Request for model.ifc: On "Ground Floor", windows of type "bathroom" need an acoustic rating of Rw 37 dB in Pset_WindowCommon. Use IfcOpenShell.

First a look at what the model holds.

```python
import ifcopenshell
import ifcopenshell.util.element

model = ifcopenshell.open("model.ifc")
print(model.schema)
storey = next(s for s in model.by_type("IfcBuildingStorey") if s.Name == "Ground Floor")
windows = [e for e in ifcopenshell.util.element.get_decomposition(storey) if e.is_a("IfcWindow")]
seen = {}
for e in windows:
    element_type = ifcopenshell.util.element.get_type(e)
    key = (element_type.Name if element_type != e and element_type else None, ifcopenshell.util.element.get_pset(e, "Pset_WindowCommon", "AcousticRating"))
    seen[key] = seen.get(key, 0) + 1
for (name, value), count in sorted(seen.items(), key=str):
    print(count, "x", name, "|", value)
```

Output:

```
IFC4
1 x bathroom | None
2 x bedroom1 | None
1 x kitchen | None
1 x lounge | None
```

```python
import ifcopenshell
import ifcopenshell.api.pset
import ifcopenshell.util.element

model = ifcopenshell.open("model.ifc")

storey = next(s for s in model.by_type("IfcBuildingStorey") if s.Name == "Ground Floor")
windows = [e for e in ifcopenshell.util.element.get_decomposition(storey) if e.is_a("IfcWindow")]

count = 0
for e in windows:
    element_type = ifcopenshell.util.element.get_type(e)
    if element_type in (None, e) or element_type.Name != "bathroom":
        continue
    # add_pset returns the element's existing set when there is one.
    pset = ifcopenshell.api.pset.add_pset(model, product=e, name="Pset_WindowCommon")
    ifcopenshell.api.pset.edit_pset(model, pset=pset, properties={"AcousticRating": "Rw 37 dB"})
    count += 1

print(count, "windows updated")

model.write("model_updated.ifc")
```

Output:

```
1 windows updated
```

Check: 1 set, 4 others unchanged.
